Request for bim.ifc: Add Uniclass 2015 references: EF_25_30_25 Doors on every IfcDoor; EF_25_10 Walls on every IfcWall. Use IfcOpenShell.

First a look at what the model holds.

```python
import ifcopenshell

model = ifcopenshell.open("bim.ifc")
print(model.schema)
print("classifications:", [c.Name for c in model.by_type("IfcClassification")])
for ifc_class in ("IfcDoor", "IfcRoof", "IfcStair", "IfcWall", "IfcWindow"):
    print(ifc_class, len(model.by_type(ifc_class)))
```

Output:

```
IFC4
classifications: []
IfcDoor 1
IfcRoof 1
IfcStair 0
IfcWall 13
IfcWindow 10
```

```python
import ifcopenshell
import ifcopenshell.api.classification

model = ifcopenshell.open("bim.ifc")

system = ifcopenshell.api.classification.add_classification(model, classification="Uniclass 2015")

codes = {
    "IfcDoor": ("EF_25_30_25", "Doors"),
    "IfcWall": ("EF_25_10", "Walls"),
}
for ifc_class, (code, name) in codes.items():
    products = model.by_type(ifc_class)
    ifcopenshell.api.classification.add_reference(
        model, products=products, classification=system, identification=code, name=name
    )
    print(code, len(products))

model.write("bim_edited.ifc")
```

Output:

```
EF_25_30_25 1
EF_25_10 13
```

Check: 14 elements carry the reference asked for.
